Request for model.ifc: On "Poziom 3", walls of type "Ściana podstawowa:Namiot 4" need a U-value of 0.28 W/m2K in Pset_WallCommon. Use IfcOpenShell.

First a look at what the model holds.

```python
import ifcopenshell
import ifcopenshell.util.element

model = ifcopenshell.open("model.ifc")
print(model.schema)
storey = next(s for s in model.by_type("IfcBuildingStorey") if s.Name == "Poziom 3")
walls = [e for e in ifcopenshell.util.element.get_decomposition(storey) if e.is_a("IfcWall")]
seen = {}
for e in walls:
    element_type = ifcopenshell.util.element.get_type(e)
    key = (element_type.Name if element_type != e and element_type else None, ifcopenshell.util.element.get_pset(e, "Pset_WallCommon", "ThermalTransmittance"))
    seen[key] = seen.get(key, 0) + 1
for (name, value), count in sorted(seen.items(), key=str):
    print(count, "x", name, "|", value)
```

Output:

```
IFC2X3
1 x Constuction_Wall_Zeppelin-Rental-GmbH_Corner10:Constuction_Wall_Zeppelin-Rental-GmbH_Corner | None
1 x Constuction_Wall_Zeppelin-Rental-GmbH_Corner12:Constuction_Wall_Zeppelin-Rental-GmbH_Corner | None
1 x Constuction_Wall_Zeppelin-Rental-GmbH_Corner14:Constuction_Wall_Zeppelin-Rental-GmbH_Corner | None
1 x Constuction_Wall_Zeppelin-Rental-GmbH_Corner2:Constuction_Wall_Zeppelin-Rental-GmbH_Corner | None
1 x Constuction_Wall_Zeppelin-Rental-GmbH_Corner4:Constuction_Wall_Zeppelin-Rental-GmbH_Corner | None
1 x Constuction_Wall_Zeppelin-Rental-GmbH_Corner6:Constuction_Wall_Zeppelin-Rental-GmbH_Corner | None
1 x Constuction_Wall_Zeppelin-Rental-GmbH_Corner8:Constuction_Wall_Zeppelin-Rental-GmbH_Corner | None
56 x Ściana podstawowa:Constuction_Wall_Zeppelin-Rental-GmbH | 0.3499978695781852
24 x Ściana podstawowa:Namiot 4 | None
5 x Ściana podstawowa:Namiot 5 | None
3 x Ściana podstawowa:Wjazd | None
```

```python
import ifcopenshell
import ifcopenshell.api.pset
import ifcopenshell.util.element

model = ifcopenshell.open("model.ifc")

storey = next(s for s in model.by_type("IfcBuildingStorey") if s.Name == "Poziom 3")
walls = [e for e in ifcopenshell.util.element.get_decomposition(storey) if e.is_a("IfcWall")]

count = 0
for e in walls:
    element_type = ifcopenshell.util.element.get_type(e)
    if element_type in (None, e) or element_type.Name != "Ściana podstawowa:Namiot 4":
        continue
    # add_pset returns the element's existing set when there is one.
    pset = ifcopenshell.api.pset.add_pset(model, product=e, name="Pset_WallCommon")
    ifcopenshell.api.pset.edit_pset(model, pset=pset, properties={"ThermalTransmittance": 0.28})
    count += 1

print(count, "walls updated")

model.write("model_updated.ifc")
```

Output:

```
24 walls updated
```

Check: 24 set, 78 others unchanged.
